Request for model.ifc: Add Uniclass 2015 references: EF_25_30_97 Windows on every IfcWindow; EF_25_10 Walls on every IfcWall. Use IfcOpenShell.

First a look at what the model holds.

```python
import ifcopenshell

model = ifcopenshell.open("model.ifc")
print(model.schema)
print("classifications:", [c.Name for c in model.by_type("IfcClassification")])
for ifc_class in ("IfcDoor", "IfcRoof", "IfcStair", "IfcWall", "IfcWindow"):
    print(ifc_class, len(model.by_type(ifc_class)))
```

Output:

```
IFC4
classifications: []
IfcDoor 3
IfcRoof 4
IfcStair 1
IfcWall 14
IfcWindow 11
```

```python
import ifcopenshell
import ifcopenshell.api.classification

model = ifcopenshell.open("model.ifc")

system = ifcopenshell.api.classification.add_classification(model, classification="Uniclass 2015")

codes = {
    "IfcWindow": ("EF_25_30_97", "Windows"),
    "IfcWall": ("EF_25_10", "Walls"),
}
for ifc_class, (code, name) in codes.items():
    products = model.by_type(ifc_class)
    ifcopenshell.api.classification.add_reference(
        model, products=products, classification=system, identification=code, name=name
    )
    print(code, len(products))

model.write("model_edited.ifc")
```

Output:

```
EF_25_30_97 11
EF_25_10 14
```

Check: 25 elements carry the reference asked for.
